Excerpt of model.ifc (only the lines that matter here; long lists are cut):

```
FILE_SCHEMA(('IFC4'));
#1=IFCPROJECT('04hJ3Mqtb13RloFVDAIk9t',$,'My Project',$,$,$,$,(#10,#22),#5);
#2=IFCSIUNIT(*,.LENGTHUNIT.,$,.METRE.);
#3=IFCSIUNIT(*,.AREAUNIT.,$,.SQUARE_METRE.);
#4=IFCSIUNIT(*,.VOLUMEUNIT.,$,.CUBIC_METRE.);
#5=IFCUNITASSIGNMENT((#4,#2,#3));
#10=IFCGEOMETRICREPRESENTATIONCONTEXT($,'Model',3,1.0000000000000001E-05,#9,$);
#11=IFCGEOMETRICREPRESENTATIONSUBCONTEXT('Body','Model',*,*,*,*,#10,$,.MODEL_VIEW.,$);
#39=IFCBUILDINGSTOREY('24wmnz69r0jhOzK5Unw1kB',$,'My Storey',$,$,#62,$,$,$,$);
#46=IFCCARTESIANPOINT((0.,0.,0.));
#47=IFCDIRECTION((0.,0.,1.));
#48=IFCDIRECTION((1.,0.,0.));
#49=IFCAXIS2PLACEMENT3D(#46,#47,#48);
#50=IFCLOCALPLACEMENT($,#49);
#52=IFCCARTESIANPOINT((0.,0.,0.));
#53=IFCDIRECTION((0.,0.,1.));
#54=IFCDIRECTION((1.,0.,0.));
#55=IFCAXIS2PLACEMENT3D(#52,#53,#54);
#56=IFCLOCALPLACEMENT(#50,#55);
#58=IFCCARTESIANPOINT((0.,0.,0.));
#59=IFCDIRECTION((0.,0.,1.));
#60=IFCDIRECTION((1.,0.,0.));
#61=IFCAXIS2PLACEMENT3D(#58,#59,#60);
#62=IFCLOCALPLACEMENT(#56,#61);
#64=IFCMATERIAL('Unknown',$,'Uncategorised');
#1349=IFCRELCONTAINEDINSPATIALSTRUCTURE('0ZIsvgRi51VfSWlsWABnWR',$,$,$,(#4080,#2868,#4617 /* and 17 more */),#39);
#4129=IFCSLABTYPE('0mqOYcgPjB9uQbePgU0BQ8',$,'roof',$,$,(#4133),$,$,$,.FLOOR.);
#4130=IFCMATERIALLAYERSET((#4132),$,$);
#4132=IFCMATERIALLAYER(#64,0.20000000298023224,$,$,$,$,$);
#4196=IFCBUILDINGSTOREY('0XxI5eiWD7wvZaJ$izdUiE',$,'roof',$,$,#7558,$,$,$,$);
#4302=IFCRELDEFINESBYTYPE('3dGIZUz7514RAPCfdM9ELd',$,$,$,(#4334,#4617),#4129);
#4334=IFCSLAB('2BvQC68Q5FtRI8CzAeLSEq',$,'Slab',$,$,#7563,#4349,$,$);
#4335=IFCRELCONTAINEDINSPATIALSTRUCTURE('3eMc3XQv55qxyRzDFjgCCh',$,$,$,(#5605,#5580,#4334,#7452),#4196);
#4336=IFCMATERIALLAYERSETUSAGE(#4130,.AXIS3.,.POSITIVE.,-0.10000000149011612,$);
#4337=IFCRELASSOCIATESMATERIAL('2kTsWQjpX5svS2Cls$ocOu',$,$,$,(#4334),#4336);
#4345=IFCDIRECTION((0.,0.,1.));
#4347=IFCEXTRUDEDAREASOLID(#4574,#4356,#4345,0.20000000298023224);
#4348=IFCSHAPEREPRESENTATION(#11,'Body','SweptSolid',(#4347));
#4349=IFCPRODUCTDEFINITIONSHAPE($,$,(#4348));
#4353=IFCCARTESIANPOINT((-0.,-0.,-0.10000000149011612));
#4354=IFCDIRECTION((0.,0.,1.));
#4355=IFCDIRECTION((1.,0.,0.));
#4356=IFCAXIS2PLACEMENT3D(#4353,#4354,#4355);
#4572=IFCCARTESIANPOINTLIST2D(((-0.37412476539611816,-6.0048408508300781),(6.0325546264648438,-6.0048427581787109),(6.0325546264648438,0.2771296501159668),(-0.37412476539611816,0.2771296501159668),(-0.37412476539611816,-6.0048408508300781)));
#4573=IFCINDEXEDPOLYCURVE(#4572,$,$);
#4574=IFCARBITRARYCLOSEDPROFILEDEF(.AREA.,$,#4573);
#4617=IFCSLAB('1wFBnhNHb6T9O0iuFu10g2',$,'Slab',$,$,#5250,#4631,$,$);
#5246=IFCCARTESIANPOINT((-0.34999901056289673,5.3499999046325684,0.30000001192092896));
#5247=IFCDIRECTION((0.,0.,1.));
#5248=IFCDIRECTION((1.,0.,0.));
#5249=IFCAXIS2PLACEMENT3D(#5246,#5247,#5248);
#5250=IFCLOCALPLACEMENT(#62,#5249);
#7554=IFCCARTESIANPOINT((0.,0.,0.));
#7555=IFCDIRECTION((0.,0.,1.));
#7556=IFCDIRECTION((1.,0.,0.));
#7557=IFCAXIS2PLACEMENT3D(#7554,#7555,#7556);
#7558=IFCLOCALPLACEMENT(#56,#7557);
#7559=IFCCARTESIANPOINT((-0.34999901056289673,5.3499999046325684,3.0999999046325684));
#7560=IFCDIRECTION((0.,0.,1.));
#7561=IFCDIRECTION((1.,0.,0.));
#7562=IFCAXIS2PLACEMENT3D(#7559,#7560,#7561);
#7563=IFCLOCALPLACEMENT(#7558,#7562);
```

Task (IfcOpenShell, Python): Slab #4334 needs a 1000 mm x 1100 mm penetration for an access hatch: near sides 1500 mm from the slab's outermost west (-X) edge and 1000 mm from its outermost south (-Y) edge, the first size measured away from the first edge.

```python
import numpy as np
import ifcopenshell
import ifcopenshell.api.feature
import ifcopenshell.api.geometry
import ifcopenshell.api.root
import ifcopenshell.geom
import ifcopenshell.util.placement
import ifcopenshell.util.representation
import ifcopenshell.util.shape
import ifcopenshell.util.unit

model = ifcopenshell.open("model.ifc")
unit_scale = ifcopenshell.util.unit.calculate_unit_scale(model)
settings = ifcopenshell.geom.settings()


def volume(element):
    """Net volume in cubic metres, openings subtracted."""
    shape = ifcopenshell.geom.create_shape(settings, element)
    return ifcopenshell.util.shape.get_volume(shape.geometry)


slab = model.by_id(4334)
before = volume(slab)

# Extent in the slab's own axes, in metres. The edges named are its -X and -Y sides.
slab_shape = ifcopenshell.geom.create_shape(settings, slab)
vertices = ifcopenshell.util.shape.get_vertices(slab_shape.geometry)
x_min, y_min, bottom = vertices.min(axis=0)
top = vertices[:, 2].max()

opening = ifcopenshell.api.root.create_entity(model, ifc_class="IfcOpeningElement", name="Access hatch opening", predefined_type="OPENING")
context = ifcopenshell.util.representation.get_context(model, "Model", "Body", "MODEL_VIEW")
width, depth = 1, 1.1
outline = [(0.0, 0.0), (width, 0.0), (width, depth), (0.0, depth), (0.0, 0.0)]
# Overshoot both faces by 50 mm so the cut is clean.
shape = ifcopenshell.api.geometry.add_slab_representation(
    model, context=context, depth=top - bottom + 0.1, polyline=outline
)
ifcopenshell.api.geometry.assign_representation(model, product=opening, representation=shape)

matrix = ifcopenshell.util.placement.get_local_placement(slab.ObjectPlacement)
matrix[:, 3] = matrix @ np.append(np.array([x_min + 1.5, y_min + 1, bottom - 0.05]) / unit_scale, 1.0)
ifcopenshell.api.geometry.edit_object_placement(model, product=opening, matrix=matrix, is_si=False)
ifcopenshell.api.feature.add_feature(model, feature=opening, element=slab)

after = volume(slab)

print(f"slab volume {before:.3f} -> {after:.3f} m3")

model.write("model_updated.ifc")
```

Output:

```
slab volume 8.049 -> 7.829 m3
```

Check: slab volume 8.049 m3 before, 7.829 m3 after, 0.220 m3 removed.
